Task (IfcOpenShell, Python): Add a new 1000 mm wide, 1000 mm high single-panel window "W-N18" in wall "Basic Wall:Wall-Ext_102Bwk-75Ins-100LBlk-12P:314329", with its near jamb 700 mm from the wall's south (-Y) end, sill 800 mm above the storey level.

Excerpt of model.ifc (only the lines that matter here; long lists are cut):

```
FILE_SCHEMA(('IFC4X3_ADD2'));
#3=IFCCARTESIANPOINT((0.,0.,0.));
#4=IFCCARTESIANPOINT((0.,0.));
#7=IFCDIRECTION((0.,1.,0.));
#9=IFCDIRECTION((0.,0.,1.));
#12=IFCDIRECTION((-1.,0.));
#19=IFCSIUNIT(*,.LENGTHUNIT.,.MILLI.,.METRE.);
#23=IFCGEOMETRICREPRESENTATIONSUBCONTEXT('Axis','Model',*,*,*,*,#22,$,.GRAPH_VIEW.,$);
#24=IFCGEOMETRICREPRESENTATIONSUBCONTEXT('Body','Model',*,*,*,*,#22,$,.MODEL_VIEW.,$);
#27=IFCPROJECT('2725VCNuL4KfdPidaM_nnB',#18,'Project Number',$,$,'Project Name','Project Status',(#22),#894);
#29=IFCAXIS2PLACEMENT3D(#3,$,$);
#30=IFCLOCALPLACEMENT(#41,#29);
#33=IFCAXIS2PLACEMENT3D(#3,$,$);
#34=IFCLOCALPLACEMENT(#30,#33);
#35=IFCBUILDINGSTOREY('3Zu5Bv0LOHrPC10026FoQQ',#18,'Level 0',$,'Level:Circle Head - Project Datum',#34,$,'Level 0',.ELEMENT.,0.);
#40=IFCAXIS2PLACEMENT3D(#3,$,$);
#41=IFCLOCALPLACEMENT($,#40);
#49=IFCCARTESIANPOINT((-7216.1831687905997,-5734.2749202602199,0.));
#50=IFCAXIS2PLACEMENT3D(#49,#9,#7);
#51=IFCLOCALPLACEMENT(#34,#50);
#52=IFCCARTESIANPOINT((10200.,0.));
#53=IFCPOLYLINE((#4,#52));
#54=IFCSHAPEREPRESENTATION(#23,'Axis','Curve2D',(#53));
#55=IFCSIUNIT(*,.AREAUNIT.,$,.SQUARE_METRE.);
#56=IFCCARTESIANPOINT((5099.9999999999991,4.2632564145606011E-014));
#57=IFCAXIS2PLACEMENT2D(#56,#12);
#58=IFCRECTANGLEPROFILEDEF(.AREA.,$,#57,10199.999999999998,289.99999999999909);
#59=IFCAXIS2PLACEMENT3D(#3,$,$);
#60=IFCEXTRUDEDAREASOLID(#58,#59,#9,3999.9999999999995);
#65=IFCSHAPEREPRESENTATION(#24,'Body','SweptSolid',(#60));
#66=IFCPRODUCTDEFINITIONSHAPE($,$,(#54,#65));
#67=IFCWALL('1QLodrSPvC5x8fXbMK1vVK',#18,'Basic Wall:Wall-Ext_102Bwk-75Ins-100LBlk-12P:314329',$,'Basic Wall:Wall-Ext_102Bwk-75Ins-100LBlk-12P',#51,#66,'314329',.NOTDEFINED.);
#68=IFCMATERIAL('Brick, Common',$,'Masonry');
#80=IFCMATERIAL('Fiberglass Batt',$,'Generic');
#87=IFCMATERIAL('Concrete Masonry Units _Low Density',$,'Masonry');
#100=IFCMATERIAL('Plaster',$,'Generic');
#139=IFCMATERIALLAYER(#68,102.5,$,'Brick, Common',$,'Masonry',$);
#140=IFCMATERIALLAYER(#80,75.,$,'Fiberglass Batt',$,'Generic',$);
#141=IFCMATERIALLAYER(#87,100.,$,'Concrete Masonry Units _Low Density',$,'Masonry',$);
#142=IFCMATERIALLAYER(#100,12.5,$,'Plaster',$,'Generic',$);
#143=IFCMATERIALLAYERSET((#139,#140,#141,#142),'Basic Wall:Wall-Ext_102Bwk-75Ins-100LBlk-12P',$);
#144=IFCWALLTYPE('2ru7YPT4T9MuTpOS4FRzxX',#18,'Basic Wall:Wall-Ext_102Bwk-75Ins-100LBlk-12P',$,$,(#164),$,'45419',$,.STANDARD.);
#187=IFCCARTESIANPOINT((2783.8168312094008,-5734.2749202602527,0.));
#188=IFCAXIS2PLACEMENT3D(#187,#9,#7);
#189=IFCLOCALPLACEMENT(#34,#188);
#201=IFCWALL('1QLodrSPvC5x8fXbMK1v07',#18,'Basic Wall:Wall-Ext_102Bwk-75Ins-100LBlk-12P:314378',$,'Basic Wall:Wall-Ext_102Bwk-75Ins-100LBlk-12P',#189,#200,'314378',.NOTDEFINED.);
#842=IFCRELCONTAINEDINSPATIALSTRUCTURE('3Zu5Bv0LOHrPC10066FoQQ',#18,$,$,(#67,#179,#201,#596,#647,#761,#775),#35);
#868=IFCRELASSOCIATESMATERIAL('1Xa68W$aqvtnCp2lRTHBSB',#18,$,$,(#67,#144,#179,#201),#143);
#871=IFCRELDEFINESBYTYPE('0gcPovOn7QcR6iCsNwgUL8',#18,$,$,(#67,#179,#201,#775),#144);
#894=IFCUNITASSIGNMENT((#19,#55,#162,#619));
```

```python
import numpy as np
import ifcopenshell
import ifcopenshell.api.feature
import ifcopenshell.api.geometry
import ifcopenshell.api.root
import ifcopenshell.api.spatial
import ifcopenshell.geom
import ifcopenshell.util.element
import ifcopenshell.util.placement
import ifcopenshell.util.representation
import ifcopenshell.util.shape
import ifcopenshell.util.unit

model = ifcopenshell.open("model.ifc")
unit_scale = ifcopenshell.util.unit.calculate_unit_scale(model)
settings = ifcopenshell.geom.settings()


def volume(element):
    """Net volume in cubic metres, openings subtracted."""
    shape = ifcopenshell.geom.create_shape(settings, element)
    return ifcopenshell.util.shape.get_volume(shape.geometry)


wall = model.by_guid("1QLodrSPvC5x8fXbMK1vVK")
storey = ifcopenshell.util.element.get_container(wall, ifc_class="IfcBuildingStorey")
context = ifcopenshell.util.representation.get_context(model, "Model", "Body", "MODEL_VIEW")
before = volume(wall)

width, height, from_end, sill = 1, 1, 0.7, 0.8  # metres

# The wall runs along its own X axis, and the end named is its -X end.
wall_shape = ifcopenshell.geom.create_shape(settings, wall)
x, y, z = ifcopenshell.util.shape.get_vertices(wall_shape.geometry).T
start = x.min() + from_end
face, thickness = float(y.min()), float(y.max() - y.min())
wall_matrix = ifcopenshell.util.placement.get_local_placement(wall.ObjectPlacement)
level = ifcopenshell.util.placement.get_local_placement(storey.ObjectPlacement)[2, 3]


def in_wall(x, y):
    """Placement at x, y metres in the wall's axes, at sill height."""
    matrix = wall_matrix.copy()
    matrix[:, 3] = wall_matrix @ np.array([x / unit_scale, y / unit_scale, 0.0, 1.0])
    matrix[2, 3] = level + sill / unit_scale
    return matrix


# Opening: a box that overshoots both wall faces by 50 mm.
opening = ifcopenshell.api.root.create_entity(model, ifc_class="IfcOpeningElement", predefined_type="OPENING")
box = ifcopenshell.api.geometry.add_wall_representation(
    model, context=context, length=width, height=height, thickness=thickness + 0.1
)
ifcopenshell.api.geometry.assign_representation(model, product=opening, representation=box)
ifcopenshell.api.geometry.edit_object_placement(model, product=opening, matrix=in_wall(start, face - 0.05), is_si=False)
ifcopenshell.api.feature.add_feature(model, feature=opening, element=wall)

window = ifcopenshell.api.root.create_entity(model, ifc_class="IfcWindow", name="W-N18", predefined_type="WINDOW")
window.OverallWidth, window.OverallHeight = width / unit_scale, height / unit_scale
window.PartitioningType = "SINGLE_PANEL"
body = ifcopenshell.api.geometry.add_window_representation(
    model,
    context=context,
    overall_width=window.OverallWidth,
    overall_height=window.OverallHeight,
    partition_type="SINGLE_PANEL",
)
ifcopenshell.api.geometry.assign_representation(model, product=window, representation=body)
ifcopenshell.api.spatial.assign_container(model, products=[window], relating_structure=storey)
ifcopenshell.api.feature.add_filling(model, opening=opening, element=window)

# Centre the window in the wall's thickness.
ifcopenshell.api.geometry.edit_object_placement(model, product=window, matrix=in_wall(start, face), is_si=False)
window_shape = ifcopenshell.geom.create_shape(settings, window)
depth = ifcopenshell.util.shape.get_vertices(window_shape.geometry)[:, 1]
offset = face + thickness / 2 - (depth.min() + depth.max()) / 2
ifcopenshell.api.geometry.edit_object_placement(model, product=window, matrix=in_wall(start, offset), is_si=False)

after = volume(wall)

print(f"wall volume {before:.3f} -> {after:.3f} m3")

model.write("model_edited.ifc")
```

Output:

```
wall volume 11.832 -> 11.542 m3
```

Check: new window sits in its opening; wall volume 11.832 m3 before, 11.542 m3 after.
